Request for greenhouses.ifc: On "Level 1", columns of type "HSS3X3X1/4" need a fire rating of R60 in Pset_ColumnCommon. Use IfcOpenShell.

First a look at what the model holds.

```python
import ifcopenshell
import ifcopenshell.util.element

model = ifcopenshell.open("greenhouses.ifc")
print(model.schema)
storey = next(s for s in model.by_type("IfcBuildingStorey") if s.Name == "Level 1")
columns = [e for e in ifcopenshell.util.element.get_decomposition(storey) if e.is_a("IfcColumn")]
seen = {}
for e in columns:
    element_type = ifcopenshell.util.element.get_type(e)
    key = (element_type.Name if element_type != e and element_type else None, ifcopenshell.util.element.get_pset(e, "Pset_ColumnCommon", "FireRating"))
    seen[key] = seen.get(key, 0) + 1
for (name, value), count in sorted(seen.items(), key=str):
    print(count, "x", name, "|", value)
```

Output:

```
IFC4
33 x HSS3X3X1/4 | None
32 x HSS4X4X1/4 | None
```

```python
import ifcopenshell
import ifcopenshell.api.pset
import ifcopenshell.util.element

model = ifcopenshell.open("greenhouses.ifc")

storey = next(s for s in model.by_type("IfcBuildingStorey") if s.Name == "Level 1")
columns = [e for e in ifcopenshell.util.element.get_decomposition(storey) if e.is_a("IfcColumn")]

count = 0
for e in columns:
    element_type = ifcopenshell.util.element.get_type(e)
    if element_type in (None, e) or element_type.Name != "HSS3X3X1/4":
        continue
    # add_pset returns the element's existing set when there is one.
    pset = ifcopenshell.api.pset.add_pset(model, product=e, name="Pset_ColumnCommon")
    ifcopenshell.api.pset.edit_pset(model, pset=pset, properties={"FireRating": "R60"})
    count += 1

print(count, "columns updated")

model.write("greenhouses-out.ifc")
```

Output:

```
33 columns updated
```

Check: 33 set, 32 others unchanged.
